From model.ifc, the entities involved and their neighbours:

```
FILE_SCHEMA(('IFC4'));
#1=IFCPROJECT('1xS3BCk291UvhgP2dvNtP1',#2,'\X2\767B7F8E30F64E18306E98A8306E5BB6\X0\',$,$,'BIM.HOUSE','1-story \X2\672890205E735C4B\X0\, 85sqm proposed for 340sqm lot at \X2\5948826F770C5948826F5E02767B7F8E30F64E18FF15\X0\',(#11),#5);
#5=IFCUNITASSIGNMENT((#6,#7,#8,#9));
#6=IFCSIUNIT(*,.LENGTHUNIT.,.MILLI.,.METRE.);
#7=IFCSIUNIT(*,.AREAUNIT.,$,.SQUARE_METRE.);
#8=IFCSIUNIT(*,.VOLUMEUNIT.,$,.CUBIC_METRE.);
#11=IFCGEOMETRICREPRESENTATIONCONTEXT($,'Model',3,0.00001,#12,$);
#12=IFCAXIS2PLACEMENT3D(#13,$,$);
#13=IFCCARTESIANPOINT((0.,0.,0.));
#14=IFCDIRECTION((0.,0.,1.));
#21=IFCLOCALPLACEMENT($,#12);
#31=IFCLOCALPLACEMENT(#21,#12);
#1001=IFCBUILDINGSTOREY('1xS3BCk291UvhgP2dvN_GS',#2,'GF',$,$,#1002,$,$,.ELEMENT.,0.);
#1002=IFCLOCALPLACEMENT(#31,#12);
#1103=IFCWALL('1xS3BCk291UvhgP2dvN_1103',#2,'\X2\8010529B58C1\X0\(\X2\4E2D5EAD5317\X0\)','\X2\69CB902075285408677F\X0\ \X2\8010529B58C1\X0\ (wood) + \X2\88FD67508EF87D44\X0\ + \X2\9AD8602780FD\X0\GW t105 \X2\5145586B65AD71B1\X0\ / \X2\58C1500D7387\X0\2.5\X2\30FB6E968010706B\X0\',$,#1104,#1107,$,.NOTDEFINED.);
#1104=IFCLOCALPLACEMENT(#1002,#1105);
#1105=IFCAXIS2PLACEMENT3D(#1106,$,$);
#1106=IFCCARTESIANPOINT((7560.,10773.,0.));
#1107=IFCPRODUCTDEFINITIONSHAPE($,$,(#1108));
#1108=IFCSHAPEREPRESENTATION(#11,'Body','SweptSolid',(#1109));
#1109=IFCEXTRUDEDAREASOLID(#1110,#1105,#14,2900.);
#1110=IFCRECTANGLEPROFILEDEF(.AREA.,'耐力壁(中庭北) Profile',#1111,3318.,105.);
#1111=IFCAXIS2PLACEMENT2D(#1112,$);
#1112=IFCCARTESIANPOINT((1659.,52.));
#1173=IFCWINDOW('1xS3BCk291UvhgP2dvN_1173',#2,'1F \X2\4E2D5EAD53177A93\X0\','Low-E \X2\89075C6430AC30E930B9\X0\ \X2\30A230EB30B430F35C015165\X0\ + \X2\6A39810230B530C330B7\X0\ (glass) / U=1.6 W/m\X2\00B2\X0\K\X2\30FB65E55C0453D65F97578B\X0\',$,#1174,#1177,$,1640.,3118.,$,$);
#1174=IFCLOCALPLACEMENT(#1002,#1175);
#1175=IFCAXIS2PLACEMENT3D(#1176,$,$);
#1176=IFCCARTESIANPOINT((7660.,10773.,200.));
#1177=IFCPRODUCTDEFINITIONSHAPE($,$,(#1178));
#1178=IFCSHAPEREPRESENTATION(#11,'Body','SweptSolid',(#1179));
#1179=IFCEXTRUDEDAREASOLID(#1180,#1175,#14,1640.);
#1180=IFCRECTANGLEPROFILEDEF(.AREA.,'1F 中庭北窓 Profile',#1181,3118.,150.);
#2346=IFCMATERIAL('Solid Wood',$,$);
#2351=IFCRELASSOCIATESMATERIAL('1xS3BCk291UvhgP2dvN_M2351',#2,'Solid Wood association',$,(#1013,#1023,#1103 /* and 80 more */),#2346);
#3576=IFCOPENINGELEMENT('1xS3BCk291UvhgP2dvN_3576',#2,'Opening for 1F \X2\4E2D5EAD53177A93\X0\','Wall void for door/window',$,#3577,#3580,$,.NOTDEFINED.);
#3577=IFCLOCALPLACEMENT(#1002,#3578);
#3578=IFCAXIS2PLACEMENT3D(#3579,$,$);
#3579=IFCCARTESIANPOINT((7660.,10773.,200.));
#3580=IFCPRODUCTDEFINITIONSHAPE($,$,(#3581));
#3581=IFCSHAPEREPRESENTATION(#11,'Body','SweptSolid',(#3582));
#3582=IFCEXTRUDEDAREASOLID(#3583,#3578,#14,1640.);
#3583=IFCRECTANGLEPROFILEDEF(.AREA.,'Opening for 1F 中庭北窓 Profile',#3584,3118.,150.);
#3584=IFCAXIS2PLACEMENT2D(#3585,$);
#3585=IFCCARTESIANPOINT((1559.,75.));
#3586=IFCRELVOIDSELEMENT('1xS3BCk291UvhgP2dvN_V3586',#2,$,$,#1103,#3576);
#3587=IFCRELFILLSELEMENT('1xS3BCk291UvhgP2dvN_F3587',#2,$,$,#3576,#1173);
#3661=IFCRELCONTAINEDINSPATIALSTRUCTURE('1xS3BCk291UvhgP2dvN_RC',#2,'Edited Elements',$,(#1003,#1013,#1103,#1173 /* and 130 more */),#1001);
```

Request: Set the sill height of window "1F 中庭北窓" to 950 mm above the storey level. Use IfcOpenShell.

```python
import numpy as np
import ifcopenshell
import ifcopenshell.api.geometry
import ifcopenshell.geom
import ifcopenshell.util.element
import ifcopenshell.util.placement
import ifcopenshell.util.shape
import ifcopenshell.util.unit

model = ifcopenshell.open("model.ifc")
unit_scale = ifcopenshell.util.unit.calculate_unit_scale(model)

window = model.by_guid("1xS3BCk291UvhgP2dvN_1173")
opening = window.FillsVoids[0].RelatingOpeningElement
storey = ifcopenshell.util.element.get_container(window, ifc_class="IfcBuildingStorey")
level = ifcopenshell.util.placement.get_local_placement(storey.ObjectPlacement)[2, 3]

# The opening's origin need not be at the sill, so measure its lowest point.
shape = ifcopenshell.geom.create_shape(ifcopenshell.geom.settings(), opening)
bottom = ifcopenshell.util.shape.get_shape_bottom_elevation(shape, shape.geometry) / unit_scale
dz = level + 0.95 / unit_scale - bottom

shift = np.array([0.0, 0.0, dz])
# The window is not placed relative to its opening, so move both.
for product in (opening, window):
    matrix = ifcopenshell.util.placement.get_local_placement(product.ObjectPlacement)
    matrix[:3, 3] += shift
    ifcopenshell.api.geometry.edit_object_placement(model, product=product, matrix=matrix, is_si=False)

print(f"moved by {dz * unit_scale:+.3f} m")

model.write("model-out.ifc")
```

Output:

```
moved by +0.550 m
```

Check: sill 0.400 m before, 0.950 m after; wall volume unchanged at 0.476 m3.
